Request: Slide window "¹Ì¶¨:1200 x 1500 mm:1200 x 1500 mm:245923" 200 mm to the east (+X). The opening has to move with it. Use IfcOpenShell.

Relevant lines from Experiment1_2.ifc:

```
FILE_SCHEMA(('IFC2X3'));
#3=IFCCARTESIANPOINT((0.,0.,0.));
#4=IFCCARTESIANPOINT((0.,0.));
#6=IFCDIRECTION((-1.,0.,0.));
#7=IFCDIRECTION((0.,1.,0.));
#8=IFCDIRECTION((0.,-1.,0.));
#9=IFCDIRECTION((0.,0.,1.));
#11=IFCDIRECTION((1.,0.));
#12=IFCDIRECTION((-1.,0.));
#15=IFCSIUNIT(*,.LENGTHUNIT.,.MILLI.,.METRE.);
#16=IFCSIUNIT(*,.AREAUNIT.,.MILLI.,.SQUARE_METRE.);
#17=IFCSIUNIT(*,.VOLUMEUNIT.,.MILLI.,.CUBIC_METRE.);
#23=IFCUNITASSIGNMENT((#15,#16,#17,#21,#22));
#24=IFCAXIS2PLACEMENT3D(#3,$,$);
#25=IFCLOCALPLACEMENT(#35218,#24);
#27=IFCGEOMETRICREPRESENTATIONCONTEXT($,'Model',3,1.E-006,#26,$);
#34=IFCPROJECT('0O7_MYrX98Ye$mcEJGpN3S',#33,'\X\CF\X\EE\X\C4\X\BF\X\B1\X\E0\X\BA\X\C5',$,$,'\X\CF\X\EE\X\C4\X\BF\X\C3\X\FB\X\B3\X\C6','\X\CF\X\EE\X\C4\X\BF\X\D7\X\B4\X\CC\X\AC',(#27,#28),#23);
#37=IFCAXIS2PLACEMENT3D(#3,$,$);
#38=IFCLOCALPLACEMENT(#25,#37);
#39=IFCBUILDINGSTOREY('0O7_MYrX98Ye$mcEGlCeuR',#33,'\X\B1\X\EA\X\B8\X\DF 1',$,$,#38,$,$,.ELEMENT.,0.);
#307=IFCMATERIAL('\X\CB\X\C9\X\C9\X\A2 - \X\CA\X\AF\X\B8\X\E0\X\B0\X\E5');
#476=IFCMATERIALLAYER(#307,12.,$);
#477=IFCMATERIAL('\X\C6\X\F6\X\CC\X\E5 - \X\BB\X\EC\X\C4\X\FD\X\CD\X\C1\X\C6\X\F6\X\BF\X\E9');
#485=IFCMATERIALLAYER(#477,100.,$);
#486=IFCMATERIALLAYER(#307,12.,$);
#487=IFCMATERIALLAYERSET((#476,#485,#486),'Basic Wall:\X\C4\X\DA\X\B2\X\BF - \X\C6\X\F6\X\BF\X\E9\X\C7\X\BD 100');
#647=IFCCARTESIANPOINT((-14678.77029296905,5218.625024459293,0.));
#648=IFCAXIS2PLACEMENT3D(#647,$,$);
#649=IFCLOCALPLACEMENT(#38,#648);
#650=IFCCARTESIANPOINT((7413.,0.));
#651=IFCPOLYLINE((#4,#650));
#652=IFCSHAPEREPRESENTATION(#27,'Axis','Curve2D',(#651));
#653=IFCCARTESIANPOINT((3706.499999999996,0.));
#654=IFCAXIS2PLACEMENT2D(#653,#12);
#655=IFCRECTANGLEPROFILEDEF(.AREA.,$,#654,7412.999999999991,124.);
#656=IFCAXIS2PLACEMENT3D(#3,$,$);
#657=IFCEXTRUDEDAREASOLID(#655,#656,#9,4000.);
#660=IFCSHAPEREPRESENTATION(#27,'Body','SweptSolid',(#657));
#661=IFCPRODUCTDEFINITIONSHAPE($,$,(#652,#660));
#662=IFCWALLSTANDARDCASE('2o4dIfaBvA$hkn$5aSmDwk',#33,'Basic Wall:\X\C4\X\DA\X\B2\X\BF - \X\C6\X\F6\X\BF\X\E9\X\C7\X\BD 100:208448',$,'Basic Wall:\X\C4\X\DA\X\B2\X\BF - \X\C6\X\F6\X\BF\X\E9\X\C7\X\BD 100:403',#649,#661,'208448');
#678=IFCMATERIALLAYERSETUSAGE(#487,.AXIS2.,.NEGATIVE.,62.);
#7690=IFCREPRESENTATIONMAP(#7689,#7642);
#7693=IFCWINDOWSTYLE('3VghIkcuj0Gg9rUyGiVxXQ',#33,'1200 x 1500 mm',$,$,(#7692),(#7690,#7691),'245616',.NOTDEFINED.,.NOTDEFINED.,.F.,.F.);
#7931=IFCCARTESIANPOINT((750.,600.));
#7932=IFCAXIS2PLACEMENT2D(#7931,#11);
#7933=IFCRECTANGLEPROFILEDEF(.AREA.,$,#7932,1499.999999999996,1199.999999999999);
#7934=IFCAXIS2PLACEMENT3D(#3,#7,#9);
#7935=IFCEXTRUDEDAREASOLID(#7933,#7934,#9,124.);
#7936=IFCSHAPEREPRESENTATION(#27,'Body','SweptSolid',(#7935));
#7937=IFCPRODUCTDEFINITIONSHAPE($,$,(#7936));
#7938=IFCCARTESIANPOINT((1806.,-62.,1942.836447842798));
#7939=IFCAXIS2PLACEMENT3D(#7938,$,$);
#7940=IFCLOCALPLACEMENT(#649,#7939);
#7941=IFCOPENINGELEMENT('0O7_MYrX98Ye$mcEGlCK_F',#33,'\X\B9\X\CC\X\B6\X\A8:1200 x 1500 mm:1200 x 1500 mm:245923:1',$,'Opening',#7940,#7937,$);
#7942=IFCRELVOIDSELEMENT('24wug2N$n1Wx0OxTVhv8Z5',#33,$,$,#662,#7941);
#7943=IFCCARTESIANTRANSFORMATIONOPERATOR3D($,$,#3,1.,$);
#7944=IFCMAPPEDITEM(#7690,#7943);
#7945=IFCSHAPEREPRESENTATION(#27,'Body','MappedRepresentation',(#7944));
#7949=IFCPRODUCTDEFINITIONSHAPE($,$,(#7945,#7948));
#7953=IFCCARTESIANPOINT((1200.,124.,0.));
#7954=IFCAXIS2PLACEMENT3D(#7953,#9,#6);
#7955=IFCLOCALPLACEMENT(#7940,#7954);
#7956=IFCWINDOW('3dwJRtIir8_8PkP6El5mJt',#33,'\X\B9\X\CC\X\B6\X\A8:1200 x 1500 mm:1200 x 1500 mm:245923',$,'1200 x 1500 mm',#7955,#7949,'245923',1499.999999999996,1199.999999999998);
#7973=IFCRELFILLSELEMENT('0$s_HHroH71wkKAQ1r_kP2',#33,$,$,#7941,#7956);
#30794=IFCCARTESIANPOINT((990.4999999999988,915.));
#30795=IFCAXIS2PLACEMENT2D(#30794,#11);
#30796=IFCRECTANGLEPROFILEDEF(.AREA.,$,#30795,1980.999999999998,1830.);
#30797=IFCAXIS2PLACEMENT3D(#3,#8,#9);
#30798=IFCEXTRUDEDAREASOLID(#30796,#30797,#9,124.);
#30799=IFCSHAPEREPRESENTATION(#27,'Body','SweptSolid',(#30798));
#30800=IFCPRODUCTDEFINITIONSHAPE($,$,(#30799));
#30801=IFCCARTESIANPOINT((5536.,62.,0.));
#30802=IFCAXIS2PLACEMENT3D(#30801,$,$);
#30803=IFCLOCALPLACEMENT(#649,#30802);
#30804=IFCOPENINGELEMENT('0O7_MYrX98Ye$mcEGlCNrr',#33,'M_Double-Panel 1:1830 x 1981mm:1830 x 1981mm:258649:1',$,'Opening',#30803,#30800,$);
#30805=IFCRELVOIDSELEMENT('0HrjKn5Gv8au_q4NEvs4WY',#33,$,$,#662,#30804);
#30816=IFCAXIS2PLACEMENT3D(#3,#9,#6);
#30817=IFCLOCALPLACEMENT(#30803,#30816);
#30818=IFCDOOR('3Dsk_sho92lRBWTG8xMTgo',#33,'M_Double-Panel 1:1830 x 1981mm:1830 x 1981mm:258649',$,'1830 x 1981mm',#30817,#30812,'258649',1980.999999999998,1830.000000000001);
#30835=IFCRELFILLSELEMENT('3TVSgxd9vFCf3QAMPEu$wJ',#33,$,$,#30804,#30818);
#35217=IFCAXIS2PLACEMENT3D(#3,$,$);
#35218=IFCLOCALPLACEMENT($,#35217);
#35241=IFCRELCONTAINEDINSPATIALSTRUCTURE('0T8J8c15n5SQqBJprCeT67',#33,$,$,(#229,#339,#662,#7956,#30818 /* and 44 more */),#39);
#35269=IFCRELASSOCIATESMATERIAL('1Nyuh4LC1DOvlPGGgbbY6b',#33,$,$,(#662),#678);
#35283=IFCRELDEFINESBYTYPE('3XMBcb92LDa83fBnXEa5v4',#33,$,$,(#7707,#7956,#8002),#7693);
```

```python
import ifcopenshell
import ifcopenshell.api.geometry
import ifcopenshell.util.placement
import ifcopenshell.util.unit

model = ifcopenshell.open("Experiment1_2.ifc")
unit_scale = ifcopenshell.util.unit.calculate_unit_scale(model)

window = model.by_guid("3dwJRtIir8_8PkP6El5mJt")
opening = window.FillsVoids[0].RelatingOpeningElement
wall = opening.VoidsElements[0].RelatingBuildingElement

wall_matrix = ifcopenshell.util.placement.get_local_placement(wall.ObjectPlacement)
shift = wall_matrix[:3, 0] * 0.2 / unit_scale
before = ifcopenshell.util.placement.get_local_placement(window.ObjectPlacement)[:3, 3].copy()

# The window is placed relative to its opening, so it follows when the opening moves.
matrix = ifcopenshell.util.placement.get_local_placement(opening.ObjectPlacement)
matrix[:3, 3] += shift
ifcopenshell.api.geometry.edit_object_placement(
    model, product=opening, matrix=matrix, is_si=False, should_transform_children=True
)

after = ifcopenshell.util.placement.get_local_placement(window.ObjectPlacement)[:3, 3]
print("window moved by", (after - before).round(3) + 0.0)

model.write("Experiment1_2-out.ifc")
```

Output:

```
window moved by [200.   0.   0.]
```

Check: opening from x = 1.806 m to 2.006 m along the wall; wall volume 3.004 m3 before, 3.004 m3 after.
